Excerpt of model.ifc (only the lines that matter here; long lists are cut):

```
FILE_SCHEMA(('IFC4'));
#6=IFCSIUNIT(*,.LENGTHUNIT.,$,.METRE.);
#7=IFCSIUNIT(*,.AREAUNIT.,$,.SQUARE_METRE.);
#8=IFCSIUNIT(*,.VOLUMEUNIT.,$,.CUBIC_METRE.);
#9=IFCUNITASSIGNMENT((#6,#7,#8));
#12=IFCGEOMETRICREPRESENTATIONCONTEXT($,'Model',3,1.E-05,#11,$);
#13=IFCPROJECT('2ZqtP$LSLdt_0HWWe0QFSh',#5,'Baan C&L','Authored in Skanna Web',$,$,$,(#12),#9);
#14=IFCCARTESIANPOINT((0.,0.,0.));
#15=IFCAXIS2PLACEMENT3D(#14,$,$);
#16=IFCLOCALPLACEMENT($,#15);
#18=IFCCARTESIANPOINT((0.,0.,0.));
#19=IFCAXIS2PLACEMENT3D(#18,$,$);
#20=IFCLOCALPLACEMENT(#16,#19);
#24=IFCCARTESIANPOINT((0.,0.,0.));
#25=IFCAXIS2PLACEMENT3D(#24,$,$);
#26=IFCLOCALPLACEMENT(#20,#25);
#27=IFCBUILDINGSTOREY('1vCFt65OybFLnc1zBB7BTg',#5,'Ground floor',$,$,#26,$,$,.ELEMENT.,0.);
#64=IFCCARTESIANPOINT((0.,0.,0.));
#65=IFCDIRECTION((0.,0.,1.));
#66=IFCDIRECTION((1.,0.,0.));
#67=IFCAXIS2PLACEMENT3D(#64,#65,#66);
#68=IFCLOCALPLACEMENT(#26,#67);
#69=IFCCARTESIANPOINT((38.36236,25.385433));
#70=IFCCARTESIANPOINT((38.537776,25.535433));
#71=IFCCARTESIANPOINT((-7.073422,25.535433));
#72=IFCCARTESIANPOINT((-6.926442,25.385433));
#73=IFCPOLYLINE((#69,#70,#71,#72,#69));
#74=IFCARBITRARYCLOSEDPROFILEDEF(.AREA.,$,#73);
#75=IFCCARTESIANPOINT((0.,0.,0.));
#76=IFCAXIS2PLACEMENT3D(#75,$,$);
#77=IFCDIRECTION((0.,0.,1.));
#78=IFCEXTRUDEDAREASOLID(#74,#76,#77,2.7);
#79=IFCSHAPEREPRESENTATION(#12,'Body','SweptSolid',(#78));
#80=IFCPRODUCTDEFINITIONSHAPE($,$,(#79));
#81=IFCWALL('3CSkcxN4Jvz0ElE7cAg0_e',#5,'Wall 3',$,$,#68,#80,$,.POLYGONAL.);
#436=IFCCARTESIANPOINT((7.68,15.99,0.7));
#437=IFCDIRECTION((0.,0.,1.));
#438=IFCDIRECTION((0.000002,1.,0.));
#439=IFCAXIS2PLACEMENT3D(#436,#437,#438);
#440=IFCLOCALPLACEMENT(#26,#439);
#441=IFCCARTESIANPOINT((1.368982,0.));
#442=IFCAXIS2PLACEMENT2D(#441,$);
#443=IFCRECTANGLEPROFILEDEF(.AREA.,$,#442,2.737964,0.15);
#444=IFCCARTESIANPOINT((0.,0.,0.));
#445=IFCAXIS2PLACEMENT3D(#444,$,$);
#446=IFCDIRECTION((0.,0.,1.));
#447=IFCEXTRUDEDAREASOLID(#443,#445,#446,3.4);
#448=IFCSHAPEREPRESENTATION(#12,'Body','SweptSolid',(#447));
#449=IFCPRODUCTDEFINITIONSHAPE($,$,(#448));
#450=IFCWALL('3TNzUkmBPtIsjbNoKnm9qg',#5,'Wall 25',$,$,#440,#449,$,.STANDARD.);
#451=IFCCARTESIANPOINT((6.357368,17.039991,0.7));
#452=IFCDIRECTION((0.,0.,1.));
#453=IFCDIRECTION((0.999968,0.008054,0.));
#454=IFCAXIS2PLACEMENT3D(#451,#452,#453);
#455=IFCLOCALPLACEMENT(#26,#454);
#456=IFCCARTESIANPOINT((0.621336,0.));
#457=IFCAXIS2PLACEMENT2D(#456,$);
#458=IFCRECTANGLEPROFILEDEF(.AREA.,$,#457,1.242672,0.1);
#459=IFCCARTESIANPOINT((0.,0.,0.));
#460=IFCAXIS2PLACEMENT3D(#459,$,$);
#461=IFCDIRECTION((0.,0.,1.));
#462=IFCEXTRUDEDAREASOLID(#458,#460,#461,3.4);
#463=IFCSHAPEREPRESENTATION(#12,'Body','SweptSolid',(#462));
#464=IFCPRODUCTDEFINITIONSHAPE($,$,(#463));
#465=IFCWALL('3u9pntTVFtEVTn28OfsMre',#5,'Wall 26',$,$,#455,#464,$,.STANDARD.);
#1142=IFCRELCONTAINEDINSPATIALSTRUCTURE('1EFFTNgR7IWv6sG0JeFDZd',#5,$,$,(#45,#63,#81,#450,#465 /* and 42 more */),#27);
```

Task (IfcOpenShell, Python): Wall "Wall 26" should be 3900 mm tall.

```python
import ifcopenshell
import ifcopenshell.geom
import ifcopenshell.util.shape
import ifcopenshell.util.unit

model = ifcopenshell.open("model.ifc")
unit_scale = ifcopenshell.util.unit.calculate_unit_scale(model)
settings = ifcopenshell.geom.settings()


def volume(element):
    """Net volume in cubic metres, openings subtracted."""
    shape = ifcopenshell.geom.create_shape(settings, element)
    return ifcopenshell.util.shape.get_volume(shape.geometry)


wall = model.by_guid("3u9pntTVFtEVTn28OfsMre")
before = volume(wall)

body = next(r for r in wall.Representation.Representations if r.RepresentationIdentifier == "Body")
solid = body.Items[0]
old_height = solid.Depth
solid.Depth = 3.9 / unit_scale
after = volume(wall)

print(f"height {old_height:g} -> {solid.Depth:g}, volume {before:.3f} -> {after:.3f} m3")

model.write("model_v2.ifc")
```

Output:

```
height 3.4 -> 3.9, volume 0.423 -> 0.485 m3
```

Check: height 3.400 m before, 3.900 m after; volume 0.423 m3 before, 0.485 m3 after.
